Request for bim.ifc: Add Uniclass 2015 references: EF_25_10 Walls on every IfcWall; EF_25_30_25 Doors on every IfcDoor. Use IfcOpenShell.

First a look at what the model holds.

```python
import ifcopenshell

model = ifcopenshell.open("bim.ifc")
print(model.schema)
print("classifications:", [c.Name for c in model.by_type("IfcClassification")])
for ifc_class in ("IfcDoor", "IfcRoof", "IfcStair", "IfcWall", "IfcWindow"):
    print(ifc_class, len(model.by_type(ifc_class)))
```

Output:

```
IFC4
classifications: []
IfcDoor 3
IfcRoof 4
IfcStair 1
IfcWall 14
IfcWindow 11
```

```python
import ifcopenshell
import ifcopenshell.api.classification

model = ifcopenshell.open("bim.ifc")

system = ifcopenshell.api.classification.add_classification(model, classification="Uniclass 2015")

codes = {
    "IfcWall": ("EF_25_10", "Walls"),
    "IfcDoor": ("EF_25_30_25", "Doors"),
}
for ifc_class, (code, name) in codes.items():
    products = model.by_type(ifc_class)
    ifcopenshell.api.classification.add_reference(
        model, products=products, classification=system, identification=code, name=name
    )
    print(code, len(products))

model.write("bim_edited.ifc")
```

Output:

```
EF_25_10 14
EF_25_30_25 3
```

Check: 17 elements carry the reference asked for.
